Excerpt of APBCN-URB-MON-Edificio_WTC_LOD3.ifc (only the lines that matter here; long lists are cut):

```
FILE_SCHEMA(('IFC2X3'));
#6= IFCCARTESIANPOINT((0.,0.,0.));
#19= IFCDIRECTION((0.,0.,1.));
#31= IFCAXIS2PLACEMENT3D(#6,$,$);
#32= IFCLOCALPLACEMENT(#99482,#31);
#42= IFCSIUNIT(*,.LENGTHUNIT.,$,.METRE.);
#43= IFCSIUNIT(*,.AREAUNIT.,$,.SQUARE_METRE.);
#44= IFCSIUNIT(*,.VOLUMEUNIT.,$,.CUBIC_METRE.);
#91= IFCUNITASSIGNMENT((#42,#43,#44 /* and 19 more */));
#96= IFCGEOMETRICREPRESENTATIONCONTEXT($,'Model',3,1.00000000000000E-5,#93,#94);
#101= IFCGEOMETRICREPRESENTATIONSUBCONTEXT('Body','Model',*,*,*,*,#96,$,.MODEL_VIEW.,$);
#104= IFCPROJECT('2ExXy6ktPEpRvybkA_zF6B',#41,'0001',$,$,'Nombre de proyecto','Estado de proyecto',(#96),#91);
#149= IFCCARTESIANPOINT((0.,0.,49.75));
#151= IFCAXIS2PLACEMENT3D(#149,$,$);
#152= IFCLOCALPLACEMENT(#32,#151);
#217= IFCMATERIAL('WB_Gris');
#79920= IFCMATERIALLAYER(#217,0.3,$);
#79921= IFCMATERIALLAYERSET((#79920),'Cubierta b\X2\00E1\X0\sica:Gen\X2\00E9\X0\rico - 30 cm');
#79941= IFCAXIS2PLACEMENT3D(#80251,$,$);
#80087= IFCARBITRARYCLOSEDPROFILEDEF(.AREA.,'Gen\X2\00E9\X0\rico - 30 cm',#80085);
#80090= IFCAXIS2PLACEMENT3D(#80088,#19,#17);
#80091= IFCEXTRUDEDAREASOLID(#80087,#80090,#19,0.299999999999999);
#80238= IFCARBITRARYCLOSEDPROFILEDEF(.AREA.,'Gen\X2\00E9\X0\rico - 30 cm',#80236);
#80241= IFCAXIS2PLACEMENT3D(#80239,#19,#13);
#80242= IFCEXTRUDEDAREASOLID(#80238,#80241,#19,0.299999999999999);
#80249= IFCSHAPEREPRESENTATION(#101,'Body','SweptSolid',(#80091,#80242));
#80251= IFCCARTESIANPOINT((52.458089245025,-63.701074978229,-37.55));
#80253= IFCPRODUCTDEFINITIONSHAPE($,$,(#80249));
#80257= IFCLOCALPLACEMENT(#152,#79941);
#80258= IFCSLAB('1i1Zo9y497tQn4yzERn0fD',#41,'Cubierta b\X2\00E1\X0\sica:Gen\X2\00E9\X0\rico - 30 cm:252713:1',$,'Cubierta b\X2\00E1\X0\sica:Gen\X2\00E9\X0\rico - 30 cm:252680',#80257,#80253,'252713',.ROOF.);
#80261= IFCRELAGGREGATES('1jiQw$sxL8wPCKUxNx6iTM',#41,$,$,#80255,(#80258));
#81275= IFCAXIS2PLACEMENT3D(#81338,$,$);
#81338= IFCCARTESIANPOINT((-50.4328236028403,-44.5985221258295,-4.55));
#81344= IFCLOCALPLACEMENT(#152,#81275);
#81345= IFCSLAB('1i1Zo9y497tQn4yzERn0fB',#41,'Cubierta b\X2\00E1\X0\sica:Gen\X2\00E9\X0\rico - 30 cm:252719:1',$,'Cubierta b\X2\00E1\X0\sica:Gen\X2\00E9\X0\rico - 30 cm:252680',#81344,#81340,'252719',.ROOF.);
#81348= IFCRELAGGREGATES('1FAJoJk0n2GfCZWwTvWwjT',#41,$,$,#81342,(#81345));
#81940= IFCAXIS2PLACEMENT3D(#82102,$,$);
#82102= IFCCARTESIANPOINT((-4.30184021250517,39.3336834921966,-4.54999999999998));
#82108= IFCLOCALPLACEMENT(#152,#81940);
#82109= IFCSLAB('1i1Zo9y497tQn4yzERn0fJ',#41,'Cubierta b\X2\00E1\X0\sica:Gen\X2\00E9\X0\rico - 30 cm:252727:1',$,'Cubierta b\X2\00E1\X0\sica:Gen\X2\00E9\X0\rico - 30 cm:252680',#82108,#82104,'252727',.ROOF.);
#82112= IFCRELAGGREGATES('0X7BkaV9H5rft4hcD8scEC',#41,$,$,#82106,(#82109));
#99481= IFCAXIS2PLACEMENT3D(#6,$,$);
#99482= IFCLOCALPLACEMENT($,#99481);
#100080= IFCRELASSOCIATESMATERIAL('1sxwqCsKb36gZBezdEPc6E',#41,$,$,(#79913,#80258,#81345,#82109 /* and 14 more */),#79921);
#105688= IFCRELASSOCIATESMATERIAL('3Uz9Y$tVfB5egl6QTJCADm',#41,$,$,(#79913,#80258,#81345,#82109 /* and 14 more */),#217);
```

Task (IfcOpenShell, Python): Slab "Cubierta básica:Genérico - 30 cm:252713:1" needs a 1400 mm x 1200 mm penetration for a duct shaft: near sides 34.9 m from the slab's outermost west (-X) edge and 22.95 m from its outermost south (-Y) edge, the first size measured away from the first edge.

```python
import numpy as np
import ifcopenshell
import ifcopenshell.api.feature
import ifcopenshell.api.geometry
import ifcopenshell.api.root
import ifcopenshell.geom
import ifcopenshell.util.placement
import ifcopenshell.util.representation
import ifcopenshell.util.shape
import ifcopenshell.util.unit

model = ifcopenshell.open("APBCN-URB-MON-Edificio_WTC_LOD3.ifc")
unit_scale = ifcopenshell.util.unit.calculate_unit_scale(model)
settings = ifcopenshell.geom.settings()


def volume(element):
    """Net volume in cubic metres, openings subtracted."""
    shape = ifcopenshell.geom.create_shape(settings, element)
    return ifcopenshell.util.shape.get_volume(shape.geometry)


slab = model.by_guid("1i1Zo9y497tQn4yzERn0fD")
before = volume(slab)

# Extent in the slab's own axes, in metres. The edges named are its -X and -Y sides.
slab_shape = ifcopenshell.geom.create_shape(settings, slab)
vertices = ifcopenshell.util.shape.get_vertices(slab_shape.geometry)
x_min, y_min, bottom = vertices.min(axis=0)
top = vertices[:, 2].max()

opening = ifcopenshell.api.root.create_entity(model, ifc_class="IfcOpeningElement", name="Duct shaft opening")
context = ifcopenshell.util.representation.get_context(model, "Model", "Body", "MODEL_VIEW")
width, depth = 1.4, 1.2
outline = [(0.0, 0.0), (width, 0.0), (width, depth), (0.0, depth), (0.0, 0.0)]
# Overshoot both faces by 50 mm so the cut is clean.
shape = ifcopenshell.api.geometry.add_slab_representation(
    model, context=context, depth=top - bottom + 0.1, polyline=outline
)
ifcopenshell.api.geometry.assign_representation(model, product=opening, representation=shape)

matrix = ifcopenshell.util.placement.get_local_placement(slab.ObjectPlacement)
matrix[:, 3] = matrix @ np.append(np.array([x_min + 34.9, y_min + 22.95, bottom - 0.05]) / unit_scale, 1.0)
ifcopenshell.api.geometry.edit_object_placement(model, product=opening, matrix=matrix, is_si=False)
ifcopenshell.api.feature.add_feature(model, feature=opening, element=slab)

after = volume(slab)

print(f"slab volume {before:.3f} -> {after:.3f} m3")

model.write("APBCN-URB-MON-Edificio_WTC_LOD3-out.ifc")
```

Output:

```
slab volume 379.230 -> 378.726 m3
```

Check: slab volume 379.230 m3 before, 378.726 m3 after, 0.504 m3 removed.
